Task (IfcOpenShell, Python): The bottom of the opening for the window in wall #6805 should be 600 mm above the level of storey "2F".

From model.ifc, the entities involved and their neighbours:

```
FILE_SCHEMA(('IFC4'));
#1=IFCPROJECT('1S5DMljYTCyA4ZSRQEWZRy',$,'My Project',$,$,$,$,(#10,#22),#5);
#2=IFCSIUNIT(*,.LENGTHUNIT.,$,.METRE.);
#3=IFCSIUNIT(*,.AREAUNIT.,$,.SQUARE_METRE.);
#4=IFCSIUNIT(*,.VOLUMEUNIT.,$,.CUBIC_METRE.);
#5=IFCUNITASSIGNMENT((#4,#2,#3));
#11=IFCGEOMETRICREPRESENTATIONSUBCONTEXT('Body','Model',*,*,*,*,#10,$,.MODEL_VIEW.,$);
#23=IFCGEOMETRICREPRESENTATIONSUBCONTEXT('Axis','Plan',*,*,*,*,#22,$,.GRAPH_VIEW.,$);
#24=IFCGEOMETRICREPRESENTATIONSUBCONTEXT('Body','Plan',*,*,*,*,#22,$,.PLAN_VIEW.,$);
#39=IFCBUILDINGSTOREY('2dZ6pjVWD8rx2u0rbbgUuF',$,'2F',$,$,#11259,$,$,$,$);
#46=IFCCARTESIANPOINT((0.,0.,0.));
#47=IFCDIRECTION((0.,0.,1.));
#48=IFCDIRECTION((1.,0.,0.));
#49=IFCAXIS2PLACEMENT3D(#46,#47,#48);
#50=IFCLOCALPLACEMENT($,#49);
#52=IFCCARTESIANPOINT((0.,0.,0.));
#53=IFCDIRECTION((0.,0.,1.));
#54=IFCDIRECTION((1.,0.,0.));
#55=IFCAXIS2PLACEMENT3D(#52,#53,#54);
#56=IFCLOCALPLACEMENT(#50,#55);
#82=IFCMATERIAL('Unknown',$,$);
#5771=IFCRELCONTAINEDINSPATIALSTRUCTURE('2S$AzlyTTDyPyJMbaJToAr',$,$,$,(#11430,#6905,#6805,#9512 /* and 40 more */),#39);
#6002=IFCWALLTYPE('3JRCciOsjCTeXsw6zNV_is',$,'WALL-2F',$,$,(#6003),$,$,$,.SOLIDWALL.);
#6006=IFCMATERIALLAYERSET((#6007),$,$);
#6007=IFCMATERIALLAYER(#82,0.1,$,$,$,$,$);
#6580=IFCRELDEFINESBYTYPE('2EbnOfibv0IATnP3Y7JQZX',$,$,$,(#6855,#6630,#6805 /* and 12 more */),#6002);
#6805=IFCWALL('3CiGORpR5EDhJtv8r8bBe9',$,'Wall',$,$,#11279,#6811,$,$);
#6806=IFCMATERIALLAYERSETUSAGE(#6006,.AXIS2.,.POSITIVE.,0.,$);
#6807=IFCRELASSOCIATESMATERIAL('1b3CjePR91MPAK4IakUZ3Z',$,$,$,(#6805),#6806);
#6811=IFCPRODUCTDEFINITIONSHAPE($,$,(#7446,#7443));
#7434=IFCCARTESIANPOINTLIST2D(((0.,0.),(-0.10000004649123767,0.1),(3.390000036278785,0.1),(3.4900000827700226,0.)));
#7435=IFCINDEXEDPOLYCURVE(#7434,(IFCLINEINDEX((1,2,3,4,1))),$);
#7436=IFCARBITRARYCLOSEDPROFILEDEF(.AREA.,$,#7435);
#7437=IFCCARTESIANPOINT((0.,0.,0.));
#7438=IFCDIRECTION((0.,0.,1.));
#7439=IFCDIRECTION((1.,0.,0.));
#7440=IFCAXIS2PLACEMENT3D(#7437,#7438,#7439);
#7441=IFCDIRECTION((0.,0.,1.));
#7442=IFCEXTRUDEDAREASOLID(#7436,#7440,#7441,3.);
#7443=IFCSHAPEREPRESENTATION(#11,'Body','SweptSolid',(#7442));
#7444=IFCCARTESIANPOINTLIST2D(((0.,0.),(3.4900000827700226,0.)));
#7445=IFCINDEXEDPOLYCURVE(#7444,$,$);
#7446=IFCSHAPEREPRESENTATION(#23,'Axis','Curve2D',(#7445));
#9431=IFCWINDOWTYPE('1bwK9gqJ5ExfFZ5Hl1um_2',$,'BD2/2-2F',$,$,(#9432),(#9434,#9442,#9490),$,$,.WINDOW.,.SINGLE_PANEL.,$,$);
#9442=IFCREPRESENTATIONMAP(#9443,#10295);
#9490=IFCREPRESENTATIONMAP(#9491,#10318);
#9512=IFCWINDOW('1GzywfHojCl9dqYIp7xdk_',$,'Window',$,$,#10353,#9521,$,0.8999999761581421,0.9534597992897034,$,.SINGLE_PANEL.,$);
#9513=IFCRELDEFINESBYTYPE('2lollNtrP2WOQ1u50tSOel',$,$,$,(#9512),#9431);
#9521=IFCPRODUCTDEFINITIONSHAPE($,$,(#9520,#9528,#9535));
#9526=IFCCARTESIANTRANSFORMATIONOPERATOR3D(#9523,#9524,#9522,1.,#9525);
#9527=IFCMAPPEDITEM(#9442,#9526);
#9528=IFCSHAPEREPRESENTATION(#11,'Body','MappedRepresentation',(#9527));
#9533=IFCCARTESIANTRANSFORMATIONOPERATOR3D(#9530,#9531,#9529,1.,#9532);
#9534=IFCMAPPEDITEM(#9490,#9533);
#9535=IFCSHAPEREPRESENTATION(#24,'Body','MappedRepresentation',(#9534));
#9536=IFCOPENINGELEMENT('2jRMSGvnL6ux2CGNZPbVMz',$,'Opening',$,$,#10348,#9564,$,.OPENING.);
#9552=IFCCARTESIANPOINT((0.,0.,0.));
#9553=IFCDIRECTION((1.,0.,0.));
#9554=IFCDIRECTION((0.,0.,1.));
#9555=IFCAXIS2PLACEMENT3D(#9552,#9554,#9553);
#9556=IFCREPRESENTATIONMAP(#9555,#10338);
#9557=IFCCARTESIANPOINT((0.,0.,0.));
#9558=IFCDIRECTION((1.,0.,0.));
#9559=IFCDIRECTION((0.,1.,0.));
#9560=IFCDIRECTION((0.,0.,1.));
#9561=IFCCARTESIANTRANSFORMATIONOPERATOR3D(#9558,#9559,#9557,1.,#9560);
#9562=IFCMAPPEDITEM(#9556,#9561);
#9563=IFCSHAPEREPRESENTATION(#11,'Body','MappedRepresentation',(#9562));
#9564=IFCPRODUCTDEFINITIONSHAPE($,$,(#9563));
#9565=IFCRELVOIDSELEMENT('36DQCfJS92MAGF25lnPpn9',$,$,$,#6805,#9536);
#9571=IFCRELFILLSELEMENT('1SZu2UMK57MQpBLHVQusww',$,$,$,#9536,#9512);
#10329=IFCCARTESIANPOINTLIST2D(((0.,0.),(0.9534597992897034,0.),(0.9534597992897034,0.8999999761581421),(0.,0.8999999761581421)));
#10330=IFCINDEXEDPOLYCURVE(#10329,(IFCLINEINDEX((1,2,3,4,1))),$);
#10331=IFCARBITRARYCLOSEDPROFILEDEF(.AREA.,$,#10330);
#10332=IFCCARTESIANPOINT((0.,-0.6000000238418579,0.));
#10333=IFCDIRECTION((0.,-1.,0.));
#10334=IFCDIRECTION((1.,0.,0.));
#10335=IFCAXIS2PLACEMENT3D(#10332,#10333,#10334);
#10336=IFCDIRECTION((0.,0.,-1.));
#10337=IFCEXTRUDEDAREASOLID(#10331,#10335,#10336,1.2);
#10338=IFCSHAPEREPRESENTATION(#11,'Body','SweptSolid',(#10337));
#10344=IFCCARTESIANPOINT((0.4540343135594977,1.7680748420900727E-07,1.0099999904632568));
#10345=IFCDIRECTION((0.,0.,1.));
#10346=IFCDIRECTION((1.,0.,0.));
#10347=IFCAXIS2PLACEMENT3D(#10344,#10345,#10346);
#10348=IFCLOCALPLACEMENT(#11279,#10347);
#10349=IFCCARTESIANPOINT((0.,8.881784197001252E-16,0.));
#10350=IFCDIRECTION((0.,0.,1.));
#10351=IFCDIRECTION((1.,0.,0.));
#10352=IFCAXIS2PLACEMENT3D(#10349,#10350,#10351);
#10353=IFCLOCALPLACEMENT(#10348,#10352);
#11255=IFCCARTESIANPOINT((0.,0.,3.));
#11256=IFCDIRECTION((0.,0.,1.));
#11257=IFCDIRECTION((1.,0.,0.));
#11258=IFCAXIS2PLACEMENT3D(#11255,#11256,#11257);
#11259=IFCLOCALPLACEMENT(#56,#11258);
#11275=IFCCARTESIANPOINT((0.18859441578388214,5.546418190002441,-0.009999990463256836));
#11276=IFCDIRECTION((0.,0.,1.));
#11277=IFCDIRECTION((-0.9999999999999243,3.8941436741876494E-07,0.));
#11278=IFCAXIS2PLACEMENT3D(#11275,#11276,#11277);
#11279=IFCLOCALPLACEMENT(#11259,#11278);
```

```python
import numpy as np
import ifcopenshell
import ifcopenshell.api.geometry
import ifcopenshell.geom
import ifcopenshell.util.element
import ifcopenshell.util.placement
import ifcopenshell.util.shape
import ifcopenshell.util.unit

model = ifcopenshell.open("model.ifc")
unit_scale = ifcopenshell.util.unit.calculate_unit_scale(model)

window = model.by_guid("1GzywfHojCl9dqYIp7xdk_")
opening = window.FillsVoids[0].RelatingOpeningElement
storey = ifcopenshell.util.element.get_container(window, ifc_class="IfcBuildingStorey")
level = ifcopenshell.util.placement.get_local_placement(storey.ObjectPlacement)[2, 3]

# The opening's origin need not be at the sill, so measure its lowest point.
shape = ifcopenshell.geom.create_shape(ifcopenshell.geom.settings(), opening)
bottom = ifcopenshell.util.shape.get_shape_bottom_elevation(shape, shape.geometry) / unit_scale
dz = level + 0.6 - bottom

shift = np.array([0.0, 0.0, dz])
# The window is placed relative to its opening, so it follows when the opening moves.
matrix = ifcopenshell.util.placement.get_local_placement(opening.ObjectPlacement)
matrix[:3, 3] += shift
ifcopenshell.api.geometry.edit_object_placement(
    model, product=opening, matrix=matrix, is_si=False, should_transform_children=True
)

print(f"moved by {dz * unit_scale:+.3f} m")

model.write("model_v2.ifc")
```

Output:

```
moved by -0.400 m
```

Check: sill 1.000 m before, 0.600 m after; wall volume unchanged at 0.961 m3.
